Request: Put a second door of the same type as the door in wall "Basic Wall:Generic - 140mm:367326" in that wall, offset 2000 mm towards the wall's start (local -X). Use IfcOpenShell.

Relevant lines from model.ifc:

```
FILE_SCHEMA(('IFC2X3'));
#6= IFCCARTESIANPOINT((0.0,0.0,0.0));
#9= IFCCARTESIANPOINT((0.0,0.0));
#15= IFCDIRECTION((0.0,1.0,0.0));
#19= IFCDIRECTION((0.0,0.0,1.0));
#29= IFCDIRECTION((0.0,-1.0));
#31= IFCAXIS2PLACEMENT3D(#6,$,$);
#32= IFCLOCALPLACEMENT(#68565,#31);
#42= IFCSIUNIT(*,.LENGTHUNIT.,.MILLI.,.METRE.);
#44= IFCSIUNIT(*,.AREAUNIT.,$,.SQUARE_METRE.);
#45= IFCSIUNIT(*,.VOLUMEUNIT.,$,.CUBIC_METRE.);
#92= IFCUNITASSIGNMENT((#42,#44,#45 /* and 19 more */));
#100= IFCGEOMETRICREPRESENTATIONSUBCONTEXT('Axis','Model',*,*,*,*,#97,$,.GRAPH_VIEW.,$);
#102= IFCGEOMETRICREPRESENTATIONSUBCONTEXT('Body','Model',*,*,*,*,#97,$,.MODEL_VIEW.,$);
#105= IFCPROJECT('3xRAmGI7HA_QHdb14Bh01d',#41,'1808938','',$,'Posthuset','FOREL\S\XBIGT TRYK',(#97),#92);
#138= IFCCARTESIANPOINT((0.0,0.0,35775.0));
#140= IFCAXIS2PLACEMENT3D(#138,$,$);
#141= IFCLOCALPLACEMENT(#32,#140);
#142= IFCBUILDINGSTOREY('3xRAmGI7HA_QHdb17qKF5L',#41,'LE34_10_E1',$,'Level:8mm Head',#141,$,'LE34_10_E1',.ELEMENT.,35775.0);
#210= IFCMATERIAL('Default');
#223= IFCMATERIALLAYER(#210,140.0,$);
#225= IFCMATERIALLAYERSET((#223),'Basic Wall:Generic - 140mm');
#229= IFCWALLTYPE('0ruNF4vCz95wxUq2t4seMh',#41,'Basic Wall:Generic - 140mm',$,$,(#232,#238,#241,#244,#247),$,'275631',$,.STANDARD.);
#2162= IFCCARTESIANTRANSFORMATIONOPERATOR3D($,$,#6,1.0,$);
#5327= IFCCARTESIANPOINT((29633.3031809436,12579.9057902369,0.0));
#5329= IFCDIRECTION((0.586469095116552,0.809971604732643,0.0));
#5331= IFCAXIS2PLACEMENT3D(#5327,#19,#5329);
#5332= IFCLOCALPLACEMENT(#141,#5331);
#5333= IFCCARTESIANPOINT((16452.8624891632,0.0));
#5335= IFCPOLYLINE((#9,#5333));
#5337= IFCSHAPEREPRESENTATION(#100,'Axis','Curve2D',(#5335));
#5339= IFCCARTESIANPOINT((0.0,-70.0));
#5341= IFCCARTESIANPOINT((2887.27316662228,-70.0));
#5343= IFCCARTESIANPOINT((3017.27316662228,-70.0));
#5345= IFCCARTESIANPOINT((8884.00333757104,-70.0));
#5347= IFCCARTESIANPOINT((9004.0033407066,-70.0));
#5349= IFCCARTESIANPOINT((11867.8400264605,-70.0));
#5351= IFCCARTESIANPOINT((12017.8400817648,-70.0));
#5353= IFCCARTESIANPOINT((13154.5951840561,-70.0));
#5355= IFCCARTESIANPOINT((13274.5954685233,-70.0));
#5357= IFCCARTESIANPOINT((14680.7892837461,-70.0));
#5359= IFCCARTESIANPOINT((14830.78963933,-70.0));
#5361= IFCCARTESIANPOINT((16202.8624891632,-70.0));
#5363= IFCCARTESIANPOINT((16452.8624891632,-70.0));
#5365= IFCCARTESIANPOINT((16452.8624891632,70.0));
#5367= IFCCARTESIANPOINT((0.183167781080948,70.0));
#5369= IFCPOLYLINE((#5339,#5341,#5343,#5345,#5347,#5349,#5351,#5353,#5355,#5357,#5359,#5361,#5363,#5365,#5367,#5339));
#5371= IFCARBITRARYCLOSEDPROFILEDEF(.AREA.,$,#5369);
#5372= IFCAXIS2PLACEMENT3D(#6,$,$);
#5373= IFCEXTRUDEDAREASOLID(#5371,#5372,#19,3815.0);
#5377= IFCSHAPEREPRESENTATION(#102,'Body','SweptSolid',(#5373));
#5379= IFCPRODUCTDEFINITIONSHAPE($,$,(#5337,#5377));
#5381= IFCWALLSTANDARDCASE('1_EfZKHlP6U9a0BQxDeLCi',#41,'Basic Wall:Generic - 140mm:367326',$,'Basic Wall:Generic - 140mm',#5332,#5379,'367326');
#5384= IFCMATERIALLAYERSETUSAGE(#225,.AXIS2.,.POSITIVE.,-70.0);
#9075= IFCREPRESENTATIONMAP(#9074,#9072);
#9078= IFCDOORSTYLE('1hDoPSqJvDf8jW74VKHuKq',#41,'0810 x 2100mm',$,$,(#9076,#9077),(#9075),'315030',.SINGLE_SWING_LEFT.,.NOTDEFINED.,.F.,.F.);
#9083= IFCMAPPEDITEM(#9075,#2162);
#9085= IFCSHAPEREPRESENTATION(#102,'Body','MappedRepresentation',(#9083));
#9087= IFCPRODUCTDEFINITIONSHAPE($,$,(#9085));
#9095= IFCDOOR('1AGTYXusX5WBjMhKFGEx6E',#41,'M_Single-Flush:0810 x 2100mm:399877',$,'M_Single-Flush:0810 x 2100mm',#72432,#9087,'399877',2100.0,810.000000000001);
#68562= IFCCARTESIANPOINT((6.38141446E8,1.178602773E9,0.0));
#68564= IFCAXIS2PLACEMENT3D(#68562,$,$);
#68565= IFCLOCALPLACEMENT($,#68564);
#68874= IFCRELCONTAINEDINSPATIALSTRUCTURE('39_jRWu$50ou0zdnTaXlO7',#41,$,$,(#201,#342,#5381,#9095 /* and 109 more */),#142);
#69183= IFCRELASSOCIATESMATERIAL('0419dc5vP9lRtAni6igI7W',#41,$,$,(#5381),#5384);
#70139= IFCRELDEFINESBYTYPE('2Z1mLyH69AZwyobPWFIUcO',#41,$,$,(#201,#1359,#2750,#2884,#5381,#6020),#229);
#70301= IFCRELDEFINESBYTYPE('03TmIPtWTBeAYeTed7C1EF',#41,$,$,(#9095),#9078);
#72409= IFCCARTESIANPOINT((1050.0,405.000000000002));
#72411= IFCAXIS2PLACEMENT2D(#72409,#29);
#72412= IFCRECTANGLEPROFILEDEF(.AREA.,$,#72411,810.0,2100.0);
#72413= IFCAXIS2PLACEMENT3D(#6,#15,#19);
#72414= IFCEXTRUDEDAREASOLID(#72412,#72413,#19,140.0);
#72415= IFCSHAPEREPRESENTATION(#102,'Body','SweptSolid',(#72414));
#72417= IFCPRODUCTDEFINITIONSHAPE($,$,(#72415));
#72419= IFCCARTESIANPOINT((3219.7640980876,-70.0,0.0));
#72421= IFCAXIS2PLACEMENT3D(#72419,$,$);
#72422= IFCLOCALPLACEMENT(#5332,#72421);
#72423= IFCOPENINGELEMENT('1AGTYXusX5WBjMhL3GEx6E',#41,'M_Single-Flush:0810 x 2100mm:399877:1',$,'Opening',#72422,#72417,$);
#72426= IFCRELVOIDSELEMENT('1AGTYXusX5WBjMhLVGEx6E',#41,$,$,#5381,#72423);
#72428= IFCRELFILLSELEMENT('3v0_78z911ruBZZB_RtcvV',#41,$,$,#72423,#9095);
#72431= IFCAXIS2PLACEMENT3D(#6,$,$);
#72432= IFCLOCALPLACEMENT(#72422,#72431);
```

```python
import ifcopenshell
import ifcopenshell.api.feature
import ifcopenshell.api.geometry
import ifcopenshell.api.root
import ifcopenshell.geom
import ifcopenshell.util.element
import ifcopenshell.util.placement
import ifcopenshell.util.shape

model = ifcopenshell.open("model.ifc")
settings = ifcopenshell.geom.settings()


def volume(element):
    """Net volume in cubic metres, openings subtracted."""
    shape = ifcopenshell.geom.create_shape(settings, element)
    return ifcopenshell.util.shape.get_volume(shape.geometry)


def reuse_history(source, copy):
    """copy_class also copies each property set's owner history, people and application; keep the originals."""
    for rel in copy.IsDefinedBy:
        if rel.is_a("IfcRelDefinesByProperties") and (history := rel.RelatingPropertyDefinition.OwnerHistory):
            rel.RelatingPropertyDefinition.OwnerHistory = source.OwnerHistory
            ifcopenshell.util.element.remove_deep2(model, history)


door = model.by_guid("1AGTYXusX5WBjMhKFGEx6E")
opening = door.FillsVoids[0].RelatingOpeningElement
wall = opening.VoidsElements[0].RelatingBuildingElement
before = volume(wall)
shift = ifcopenshell.util.placement.get_local_placement(wall.ObjectPlacement)[:3, 0] * -2000.0

# copy_class copies the void relationship, type, container and properties, but no geometry.
new_opening = ifcopenshell.api.root.copy_class(model, product=opening)
new_opening.Representation = ifcopenshell.util.element.copy_deep(
    model, opening.Representation, exclude=["IfcGeometricRepresentationContext", "IfcRepresentationMap"]
)
new_opening.Name = "M_Single-Flush:0810 x 2100mm"
new_door = ifcopenshell.api.root.copy_class(model, product=door)
new_door.Representation = ifcopenshell.util.element.copy_deep(
    model, door.Representation, exclude=["IfcGeometricRepresentationContext", "IfcRepresentationMap"]
)
new_door.Name = "M_Single-Flush:0810 x 2100mm"
new_door.Tag = None
reuse_history(door, new_door)
fills = ifcopenshell.api.feature.add_filling(model, opening=new_opening, element=new_door)
fills.OwnerHistory = new_door.OwnerHistory  # required in IFC2X3

for old, new in ((opening, new_opening), (door, new_door)):
    matrix = ifcopenshell.util.placement.get_local_placement(old.ObjectPlacement)
    matrix[:3, 3] += shift
    ifcopenshell.api.geometry.edit_object_placement(model, product=new, matrix=matrix, is_si=False)

after = volume(wall)

print(f"wall volume {before:.3f} -> {after:.3f} m3")

model.write("model_rev.ifc")
```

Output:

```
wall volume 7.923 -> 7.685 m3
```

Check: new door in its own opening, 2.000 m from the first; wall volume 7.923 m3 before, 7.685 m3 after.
